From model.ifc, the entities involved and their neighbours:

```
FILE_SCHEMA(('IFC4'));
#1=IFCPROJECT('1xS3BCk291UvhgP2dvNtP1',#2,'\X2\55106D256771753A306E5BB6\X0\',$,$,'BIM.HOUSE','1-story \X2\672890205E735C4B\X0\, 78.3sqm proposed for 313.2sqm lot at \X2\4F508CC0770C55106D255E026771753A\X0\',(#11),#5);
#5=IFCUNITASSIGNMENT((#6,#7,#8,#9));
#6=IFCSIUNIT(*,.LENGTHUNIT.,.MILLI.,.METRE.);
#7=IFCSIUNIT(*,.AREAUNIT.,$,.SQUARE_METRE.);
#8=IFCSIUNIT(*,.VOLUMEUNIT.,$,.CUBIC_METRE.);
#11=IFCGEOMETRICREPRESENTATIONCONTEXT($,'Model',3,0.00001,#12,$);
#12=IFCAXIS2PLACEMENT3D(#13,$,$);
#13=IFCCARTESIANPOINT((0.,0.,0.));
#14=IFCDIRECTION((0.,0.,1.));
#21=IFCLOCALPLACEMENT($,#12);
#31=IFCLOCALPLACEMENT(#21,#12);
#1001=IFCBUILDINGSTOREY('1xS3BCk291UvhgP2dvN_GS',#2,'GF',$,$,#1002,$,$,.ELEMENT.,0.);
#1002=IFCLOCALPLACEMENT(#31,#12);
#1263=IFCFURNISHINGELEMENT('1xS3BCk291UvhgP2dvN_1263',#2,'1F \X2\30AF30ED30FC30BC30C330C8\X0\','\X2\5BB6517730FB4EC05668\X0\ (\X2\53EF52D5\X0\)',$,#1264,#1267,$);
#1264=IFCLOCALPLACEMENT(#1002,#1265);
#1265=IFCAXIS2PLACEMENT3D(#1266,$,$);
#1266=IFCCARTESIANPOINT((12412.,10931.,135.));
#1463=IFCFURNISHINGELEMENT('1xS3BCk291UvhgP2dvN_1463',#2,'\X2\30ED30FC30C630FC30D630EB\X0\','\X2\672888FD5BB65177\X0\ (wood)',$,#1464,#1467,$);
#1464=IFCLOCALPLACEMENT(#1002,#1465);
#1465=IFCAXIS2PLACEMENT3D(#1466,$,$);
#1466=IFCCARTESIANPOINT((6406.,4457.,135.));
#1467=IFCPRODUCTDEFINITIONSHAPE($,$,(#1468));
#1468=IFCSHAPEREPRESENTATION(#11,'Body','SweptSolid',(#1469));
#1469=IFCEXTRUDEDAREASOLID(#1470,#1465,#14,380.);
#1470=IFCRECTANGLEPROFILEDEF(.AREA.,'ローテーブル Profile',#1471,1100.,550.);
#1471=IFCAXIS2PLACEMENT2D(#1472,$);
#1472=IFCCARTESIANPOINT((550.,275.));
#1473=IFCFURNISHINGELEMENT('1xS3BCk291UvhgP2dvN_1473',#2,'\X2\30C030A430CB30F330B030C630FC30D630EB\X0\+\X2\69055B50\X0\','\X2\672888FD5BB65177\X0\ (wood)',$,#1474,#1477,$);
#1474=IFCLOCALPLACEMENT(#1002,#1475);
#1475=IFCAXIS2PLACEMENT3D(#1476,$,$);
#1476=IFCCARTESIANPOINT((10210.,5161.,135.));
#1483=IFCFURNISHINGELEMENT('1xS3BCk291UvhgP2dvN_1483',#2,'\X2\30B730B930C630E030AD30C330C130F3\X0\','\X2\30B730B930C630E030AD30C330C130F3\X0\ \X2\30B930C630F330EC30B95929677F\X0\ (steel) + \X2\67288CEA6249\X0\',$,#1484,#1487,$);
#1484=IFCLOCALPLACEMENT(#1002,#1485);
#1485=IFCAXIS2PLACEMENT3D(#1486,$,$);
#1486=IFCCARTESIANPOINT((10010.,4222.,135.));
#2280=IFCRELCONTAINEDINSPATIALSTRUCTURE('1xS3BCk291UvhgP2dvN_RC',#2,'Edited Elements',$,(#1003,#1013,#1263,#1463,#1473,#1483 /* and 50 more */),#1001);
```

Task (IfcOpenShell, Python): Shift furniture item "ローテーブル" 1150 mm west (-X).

```python
import ifcopenshell
import ifcopenshell.api.geometry
import ifcopenshell.util.placement
import ifcopenshell.util.unit

model = ifcopenshell.open("model.ifc")
unit_scale = ifcopenshell.util.unit.calculate_unit_scale(model)

item = model.by_guid("1xS3BCk291UvhgP2dvN_1463")
matrix = ifcopenshell.util.placement.get_local_placement(item.ObjectPlacement)
matrix[0, 3] -= 1.15 / unit_scale
ifcopenshell.api.geometry.edit_object_placement(model, product=item, matrix=matrix, is_si=False)

print(ifcopenshell.util.placement.get_local_placement(item.ObjectPlacement).round(3) + 0.0)

model.write("model_v2.ifc")
```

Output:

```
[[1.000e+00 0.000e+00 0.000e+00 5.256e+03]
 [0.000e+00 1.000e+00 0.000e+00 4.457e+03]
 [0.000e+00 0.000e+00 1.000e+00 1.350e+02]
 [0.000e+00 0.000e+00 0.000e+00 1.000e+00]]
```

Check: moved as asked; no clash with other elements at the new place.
